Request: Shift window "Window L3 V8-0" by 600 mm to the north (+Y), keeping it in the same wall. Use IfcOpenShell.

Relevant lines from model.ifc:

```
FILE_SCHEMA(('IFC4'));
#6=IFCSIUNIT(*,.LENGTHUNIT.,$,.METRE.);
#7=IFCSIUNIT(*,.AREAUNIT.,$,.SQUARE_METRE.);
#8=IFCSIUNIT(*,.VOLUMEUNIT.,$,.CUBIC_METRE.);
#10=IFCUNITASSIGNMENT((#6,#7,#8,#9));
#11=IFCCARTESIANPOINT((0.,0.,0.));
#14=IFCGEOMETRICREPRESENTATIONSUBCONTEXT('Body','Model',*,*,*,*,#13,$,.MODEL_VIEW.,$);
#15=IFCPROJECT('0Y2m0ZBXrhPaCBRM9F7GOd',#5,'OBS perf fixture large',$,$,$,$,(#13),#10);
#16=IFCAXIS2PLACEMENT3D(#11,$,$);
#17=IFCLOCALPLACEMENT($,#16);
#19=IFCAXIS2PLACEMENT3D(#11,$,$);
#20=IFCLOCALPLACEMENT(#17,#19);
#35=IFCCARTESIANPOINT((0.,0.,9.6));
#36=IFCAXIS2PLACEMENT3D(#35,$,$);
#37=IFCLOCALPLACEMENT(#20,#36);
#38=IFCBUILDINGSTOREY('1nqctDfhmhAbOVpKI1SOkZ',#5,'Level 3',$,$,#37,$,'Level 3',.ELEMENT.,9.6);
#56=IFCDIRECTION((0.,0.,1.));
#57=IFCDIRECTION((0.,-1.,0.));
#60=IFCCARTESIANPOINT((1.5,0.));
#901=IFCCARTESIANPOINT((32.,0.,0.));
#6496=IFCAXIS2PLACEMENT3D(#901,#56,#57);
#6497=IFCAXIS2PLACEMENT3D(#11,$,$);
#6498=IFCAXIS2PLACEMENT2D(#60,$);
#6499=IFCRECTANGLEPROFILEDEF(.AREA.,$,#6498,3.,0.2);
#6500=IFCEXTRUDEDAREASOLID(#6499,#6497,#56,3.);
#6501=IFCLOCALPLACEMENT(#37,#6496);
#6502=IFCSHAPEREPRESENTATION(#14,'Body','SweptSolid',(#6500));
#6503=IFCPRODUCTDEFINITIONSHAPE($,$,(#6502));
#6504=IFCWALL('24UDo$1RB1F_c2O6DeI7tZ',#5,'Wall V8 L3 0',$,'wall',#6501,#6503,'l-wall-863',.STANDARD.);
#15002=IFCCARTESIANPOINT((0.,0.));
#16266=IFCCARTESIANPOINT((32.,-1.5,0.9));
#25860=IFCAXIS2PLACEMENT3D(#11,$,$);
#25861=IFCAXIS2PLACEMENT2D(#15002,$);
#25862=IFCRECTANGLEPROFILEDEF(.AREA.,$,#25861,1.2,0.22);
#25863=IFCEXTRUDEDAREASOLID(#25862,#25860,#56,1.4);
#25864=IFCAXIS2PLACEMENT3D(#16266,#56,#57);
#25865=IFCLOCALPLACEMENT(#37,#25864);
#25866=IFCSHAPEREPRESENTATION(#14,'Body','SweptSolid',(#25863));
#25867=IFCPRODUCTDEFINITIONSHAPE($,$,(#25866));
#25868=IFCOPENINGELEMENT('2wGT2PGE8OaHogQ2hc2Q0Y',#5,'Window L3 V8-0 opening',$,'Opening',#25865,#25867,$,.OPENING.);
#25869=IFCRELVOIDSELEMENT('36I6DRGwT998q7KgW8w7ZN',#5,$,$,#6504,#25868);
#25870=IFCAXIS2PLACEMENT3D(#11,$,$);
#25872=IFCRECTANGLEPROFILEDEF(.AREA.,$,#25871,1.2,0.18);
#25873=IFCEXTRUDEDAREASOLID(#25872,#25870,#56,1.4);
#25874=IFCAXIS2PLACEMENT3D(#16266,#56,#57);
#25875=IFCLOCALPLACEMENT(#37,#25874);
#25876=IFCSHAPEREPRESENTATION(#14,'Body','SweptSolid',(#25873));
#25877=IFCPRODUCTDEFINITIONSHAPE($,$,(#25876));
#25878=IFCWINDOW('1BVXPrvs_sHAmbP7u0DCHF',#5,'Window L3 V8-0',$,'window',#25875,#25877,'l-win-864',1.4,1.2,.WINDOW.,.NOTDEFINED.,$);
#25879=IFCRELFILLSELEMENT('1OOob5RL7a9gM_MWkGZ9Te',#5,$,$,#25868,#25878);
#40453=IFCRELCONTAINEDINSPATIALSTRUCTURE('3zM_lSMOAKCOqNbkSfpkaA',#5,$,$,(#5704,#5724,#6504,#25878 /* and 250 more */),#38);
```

```python
import ifcopenshell
import ifcopenshell.api.geometry
import ifcopenshell.util.placement

model = ifcopenshell.open("model.ifc")

window = model.by_guid("1BVXPrvs_sHAmbP7u0DCHF")
opening = window.FillsVoids[0].RelatingOpeningElement
wall = opening.VoidsElements[0].RelatingBuildingElement

wall_matrix = ifcopenshell.util.placement.get_local_placement(wall.ObjectPlacement)
shift = wall_matrix[:3, 0] * -0.6
before = ifcopenshell.util.placement.get_local_placement(window.ObjectPlacement)[:3, 3].copy()

# The window is not placed relative to its opening, so move both.
for product in (opening, window):
    matrix = ifcopenshell.util.placement.get_local_placement(product.ObjectPlacement)
    matrix[:3, 3] += shift
    ifcopenshell.api.geometry.edit_object_placement(model, product=product, matrix=matrix, is_si=False)

after = ifcopenshell.util.placement.get_local_placement(window.ObjectPlacement)[:3, 3]
print("window moved by", (after - before).round(3) + 0.0)

model.write("model-out.ifc")
```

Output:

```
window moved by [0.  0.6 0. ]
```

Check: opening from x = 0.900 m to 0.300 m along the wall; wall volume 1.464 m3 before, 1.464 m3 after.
